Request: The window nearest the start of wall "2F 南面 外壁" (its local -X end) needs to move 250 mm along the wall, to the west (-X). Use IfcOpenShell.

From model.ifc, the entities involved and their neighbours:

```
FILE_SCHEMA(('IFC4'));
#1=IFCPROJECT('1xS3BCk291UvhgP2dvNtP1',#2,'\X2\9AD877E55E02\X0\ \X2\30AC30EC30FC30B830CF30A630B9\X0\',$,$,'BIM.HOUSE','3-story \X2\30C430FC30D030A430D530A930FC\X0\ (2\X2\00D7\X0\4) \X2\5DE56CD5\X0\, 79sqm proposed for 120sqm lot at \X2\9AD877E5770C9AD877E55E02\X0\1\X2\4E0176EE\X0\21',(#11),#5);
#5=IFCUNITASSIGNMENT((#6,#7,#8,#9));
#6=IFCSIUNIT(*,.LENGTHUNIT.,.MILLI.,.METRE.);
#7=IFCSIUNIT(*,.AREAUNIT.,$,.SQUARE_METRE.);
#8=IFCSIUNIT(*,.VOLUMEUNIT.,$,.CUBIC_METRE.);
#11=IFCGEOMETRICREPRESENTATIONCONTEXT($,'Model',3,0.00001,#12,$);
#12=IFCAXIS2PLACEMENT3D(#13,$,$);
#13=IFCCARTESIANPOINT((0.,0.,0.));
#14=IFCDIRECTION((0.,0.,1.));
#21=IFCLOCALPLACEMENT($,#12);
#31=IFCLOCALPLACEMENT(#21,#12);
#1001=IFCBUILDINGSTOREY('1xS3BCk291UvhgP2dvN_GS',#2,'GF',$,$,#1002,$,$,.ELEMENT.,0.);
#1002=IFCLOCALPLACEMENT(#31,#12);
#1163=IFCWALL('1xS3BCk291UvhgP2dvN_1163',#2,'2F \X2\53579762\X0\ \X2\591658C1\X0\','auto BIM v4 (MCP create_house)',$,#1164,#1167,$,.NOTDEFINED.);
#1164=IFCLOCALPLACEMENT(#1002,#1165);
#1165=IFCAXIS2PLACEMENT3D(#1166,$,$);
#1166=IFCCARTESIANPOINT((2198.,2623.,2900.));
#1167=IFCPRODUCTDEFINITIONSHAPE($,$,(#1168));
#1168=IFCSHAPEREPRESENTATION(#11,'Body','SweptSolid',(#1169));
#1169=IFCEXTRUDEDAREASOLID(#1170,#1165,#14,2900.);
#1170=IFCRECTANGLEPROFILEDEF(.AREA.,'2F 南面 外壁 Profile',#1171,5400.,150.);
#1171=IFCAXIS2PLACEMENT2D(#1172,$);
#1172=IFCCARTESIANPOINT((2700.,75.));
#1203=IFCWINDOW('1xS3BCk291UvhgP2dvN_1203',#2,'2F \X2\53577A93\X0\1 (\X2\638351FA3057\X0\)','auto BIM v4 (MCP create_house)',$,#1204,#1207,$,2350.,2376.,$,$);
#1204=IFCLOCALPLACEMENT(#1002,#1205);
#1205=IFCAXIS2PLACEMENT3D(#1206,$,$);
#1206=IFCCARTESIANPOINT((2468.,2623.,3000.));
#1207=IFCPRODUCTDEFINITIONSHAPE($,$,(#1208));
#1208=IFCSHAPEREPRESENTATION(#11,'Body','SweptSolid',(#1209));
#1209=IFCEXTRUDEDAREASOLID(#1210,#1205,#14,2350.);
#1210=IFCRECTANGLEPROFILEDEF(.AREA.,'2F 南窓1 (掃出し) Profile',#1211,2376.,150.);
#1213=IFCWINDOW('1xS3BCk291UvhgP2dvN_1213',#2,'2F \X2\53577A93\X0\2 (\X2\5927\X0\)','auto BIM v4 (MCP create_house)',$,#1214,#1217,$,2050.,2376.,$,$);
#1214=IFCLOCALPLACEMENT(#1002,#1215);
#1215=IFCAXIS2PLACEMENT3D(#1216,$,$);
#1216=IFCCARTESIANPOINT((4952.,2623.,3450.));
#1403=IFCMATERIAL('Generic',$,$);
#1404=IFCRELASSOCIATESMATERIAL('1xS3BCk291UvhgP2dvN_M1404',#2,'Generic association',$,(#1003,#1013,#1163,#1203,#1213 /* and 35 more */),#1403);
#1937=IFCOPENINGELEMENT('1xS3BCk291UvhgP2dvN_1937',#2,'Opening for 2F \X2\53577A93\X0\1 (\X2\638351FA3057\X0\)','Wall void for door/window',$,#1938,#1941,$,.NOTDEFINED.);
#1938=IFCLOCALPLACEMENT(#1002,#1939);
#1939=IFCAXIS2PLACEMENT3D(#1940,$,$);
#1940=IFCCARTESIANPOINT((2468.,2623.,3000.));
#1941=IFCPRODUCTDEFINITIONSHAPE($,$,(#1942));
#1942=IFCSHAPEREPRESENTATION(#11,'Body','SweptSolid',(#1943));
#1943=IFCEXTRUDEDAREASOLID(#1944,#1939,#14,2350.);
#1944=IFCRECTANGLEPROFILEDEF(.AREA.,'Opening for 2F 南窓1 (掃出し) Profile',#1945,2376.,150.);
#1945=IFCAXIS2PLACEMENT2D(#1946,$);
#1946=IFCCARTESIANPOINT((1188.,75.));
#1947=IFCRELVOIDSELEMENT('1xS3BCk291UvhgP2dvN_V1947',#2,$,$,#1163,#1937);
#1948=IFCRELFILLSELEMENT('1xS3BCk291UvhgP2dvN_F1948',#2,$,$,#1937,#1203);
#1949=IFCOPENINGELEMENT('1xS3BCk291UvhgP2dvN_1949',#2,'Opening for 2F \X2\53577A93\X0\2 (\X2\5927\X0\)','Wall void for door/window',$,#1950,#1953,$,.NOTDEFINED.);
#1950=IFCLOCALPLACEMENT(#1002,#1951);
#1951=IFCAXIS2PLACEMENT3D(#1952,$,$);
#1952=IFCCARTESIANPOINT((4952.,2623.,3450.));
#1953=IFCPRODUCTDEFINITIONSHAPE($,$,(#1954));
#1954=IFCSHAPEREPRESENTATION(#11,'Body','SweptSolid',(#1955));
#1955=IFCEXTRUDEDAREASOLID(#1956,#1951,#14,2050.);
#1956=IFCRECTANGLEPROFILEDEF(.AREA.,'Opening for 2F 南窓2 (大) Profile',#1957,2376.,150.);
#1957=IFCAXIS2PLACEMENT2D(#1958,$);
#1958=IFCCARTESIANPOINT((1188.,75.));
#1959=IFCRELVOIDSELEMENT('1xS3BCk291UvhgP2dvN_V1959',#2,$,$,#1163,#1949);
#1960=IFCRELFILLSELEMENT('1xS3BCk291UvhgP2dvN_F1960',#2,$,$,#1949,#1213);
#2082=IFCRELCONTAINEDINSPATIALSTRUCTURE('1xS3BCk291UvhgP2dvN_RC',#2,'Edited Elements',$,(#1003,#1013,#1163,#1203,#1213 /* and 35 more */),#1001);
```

```python
import ifcopenshell
import ifcopenshell.api.geometry
import ifcopenshell.util.placement
import ifcopenshell.util.unit

model = ifcopenshell.open("model.ifc")
unit_scale = ifcopenshell.util.unit.calculate_unit_scale(model)

window = model.by_guid("1xS3BCk291UvhgP2dvN_1203")
opening = window.FillsVoids[0].RelatingOpeningElement
wall = opening.VoidsElements[0].RelatingBuildingElement

wall_matrix = ifcopenshell.util.placement.get_local_placement(wall.ObjectPlacement)
shift = wall_matrix[:3, 0] * -0.25 / unit_scale
before = ifcopenshell.util.placement.get_local_placement(window.ObjectPlacement)[:3, 3].copy()

# The window is not placed relative to its opening, so move both.
for product in (opening, window):
    matrix = ifcopenshell.util.placement.get_local_placement(product.ObjectPlacement)
    matrix[:3, 3] += shift
    ifcopenshell.api.geometry.edit_object_placement(model, product=product, matrix=matrix, is_si=False)

after = ifcopenshell.util.placement.get_local_placement(window.ObjectPlacement)[:3, 3]
print("window moved by", (after - before).round(3) + 0.0)

model.write("model_edited.ifc")
```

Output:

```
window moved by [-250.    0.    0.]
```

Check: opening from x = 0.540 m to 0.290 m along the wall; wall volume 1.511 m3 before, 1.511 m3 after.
